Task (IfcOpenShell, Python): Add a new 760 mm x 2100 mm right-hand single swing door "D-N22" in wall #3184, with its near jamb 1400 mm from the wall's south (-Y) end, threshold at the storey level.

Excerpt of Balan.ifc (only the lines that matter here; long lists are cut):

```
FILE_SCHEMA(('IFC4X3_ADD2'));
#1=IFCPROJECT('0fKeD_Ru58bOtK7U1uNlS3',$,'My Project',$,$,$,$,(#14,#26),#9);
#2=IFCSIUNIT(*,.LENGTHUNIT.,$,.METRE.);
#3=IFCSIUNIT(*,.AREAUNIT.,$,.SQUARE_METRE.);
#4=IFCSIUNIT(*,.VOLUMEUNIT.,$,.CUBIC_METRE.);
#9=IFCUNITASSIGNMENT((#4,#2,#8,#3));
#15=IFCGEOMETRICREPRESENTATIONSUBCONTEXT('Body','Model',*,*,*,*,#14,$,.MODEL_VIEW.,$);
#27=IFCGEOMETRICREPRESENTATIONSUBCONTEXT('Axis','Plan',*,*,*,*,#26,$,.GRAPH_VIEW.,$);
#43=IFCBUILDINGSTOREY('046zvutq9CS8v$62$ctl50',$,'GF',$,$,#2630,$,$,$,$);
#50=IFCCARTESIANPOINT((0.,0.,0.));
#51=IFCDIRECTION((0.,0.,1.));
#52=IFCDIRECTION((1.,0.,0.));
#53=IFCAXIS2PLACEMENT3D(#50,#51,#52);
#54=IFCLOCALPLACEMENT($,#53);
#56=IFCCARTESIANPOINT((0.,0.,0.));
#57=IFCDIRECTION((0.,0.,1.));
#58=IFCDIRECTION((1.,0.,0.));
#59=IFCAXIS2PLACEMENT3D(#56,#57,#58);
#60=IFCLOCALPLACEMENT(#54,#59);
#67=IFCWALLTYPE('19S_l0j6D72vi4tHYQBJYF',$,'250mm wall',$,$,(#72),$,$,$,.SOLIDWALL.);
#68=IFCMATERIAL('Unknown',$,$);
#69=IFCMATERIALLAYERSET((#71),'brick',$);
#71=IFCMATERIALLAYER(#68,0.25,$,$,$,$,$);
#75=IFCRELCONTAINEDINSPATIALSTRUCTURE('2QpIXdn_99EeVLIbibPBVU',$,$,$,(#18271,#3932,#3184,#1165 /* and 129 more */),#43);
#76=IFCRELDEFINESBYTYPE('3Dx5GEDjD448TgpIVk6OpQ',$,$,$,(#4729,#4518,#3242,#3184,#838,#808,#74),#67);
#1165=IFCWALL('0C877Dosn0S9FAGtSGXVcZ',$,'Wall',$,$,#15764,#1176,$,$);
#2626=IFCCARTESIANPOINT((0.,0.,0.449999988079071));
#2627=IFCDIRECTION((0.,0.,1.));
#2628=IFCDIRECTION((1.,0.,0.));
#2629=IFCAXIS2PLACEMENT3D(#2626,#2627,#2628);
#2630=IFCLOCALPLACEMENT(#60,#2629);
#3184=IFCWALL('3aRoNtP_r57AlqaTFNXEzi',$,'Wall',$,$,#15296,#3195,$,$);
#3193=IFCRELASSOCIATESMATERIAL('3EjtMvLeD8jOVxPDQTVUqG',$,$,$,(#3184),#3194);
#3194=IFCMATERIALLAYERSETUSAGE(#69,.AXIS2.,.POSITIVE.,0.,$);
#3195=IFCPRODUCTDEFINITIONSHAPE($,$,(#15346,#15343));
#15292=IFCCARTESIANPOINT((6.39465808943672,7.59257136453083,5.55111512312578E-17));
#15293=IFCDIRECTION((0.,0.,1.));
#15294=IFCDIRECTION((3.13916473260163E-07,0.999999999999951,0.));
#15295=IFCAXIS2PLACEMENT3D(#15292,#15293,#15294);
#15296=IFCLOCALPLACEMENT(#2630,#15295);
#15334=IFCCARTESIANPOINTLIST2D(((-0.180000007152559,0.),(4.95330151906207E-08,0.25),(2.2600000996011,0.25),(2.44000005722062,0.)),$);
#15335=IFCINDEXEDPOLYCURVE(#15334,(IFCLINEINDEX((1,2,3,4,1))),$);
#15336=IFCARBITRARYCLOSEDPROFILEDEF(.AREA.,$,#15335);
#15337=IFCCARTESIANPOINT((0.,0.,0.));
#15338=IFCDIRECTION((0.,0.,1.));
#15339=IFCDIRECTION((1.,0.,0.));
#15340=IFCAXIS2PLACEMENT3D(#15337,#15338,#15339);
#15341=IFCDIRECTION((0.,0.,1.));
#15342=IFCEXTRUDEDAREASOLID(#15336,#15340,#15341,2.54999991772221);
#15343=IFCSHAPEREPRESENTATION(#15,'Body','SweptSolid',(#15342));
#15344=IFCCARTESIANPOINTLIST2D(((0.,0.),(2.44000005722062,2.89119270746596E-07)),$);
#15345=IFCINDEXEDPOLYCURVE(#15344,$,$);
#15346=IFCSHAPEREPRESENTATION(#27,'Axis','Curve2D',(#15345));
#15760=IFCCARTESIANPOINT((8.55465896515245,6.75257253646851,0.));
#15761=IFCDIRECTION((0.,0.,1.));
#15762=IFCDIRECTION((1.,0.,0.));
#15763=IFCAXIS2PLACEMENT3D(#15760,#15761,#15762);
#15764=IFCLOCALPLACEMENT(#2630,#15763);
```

```python
import numpy as np
import ifcopenshell
import ifcopenshell.api.feature
import ifcopenshell.api.geometry
import ifcopenshell.api.root
import ifcopenshell.api.spatial
import ifcopenshell.geom
import ifcopenshell.util.element
import ifcopenshell.util.placement
import ifcopenshell.util.representation
import ifcopenshell.util.shape
import ifcopenshell.util.unit

model = ifcopenshell.open("Balan.ifc")
unit_scale = ifcopenshell.util.unit.calculate_unit_scale(model)
settings = ifcopenshell.geom.settings()


def volume(element):
    """Net volume in cubic metres, openings subtracted."""
    shape = ifcopenshell.geom.create_shape(settings, element)
    return ifcopenshell.util.shape.get_volume(shape.geometry)


wall = model.by_guid("3aRoNtP_r57AlqaTFNXEzi")
storey = ifcopenshell.util.element.get_container(wall, ifc_class="IfcBuildingStorey")
context = ifcopenshell.util.representation.get_context(model, "Model", "Body", "MODEL_VIEW")
before = volume(wall)

width, height, from_end, sill = 0.76, 2.1, 1.4, 0.0  # metres

# The wall runs along its own X axis, and the end named is its -X end.
wall_shape = ifcopenshell.geom.create_shape(settings, wall)
x, y, z = ifcopenshell.util.shape.get_vertices(wall_shape.geometry).T
start = x.min() + from_end
face, thickness = float(y.min()), float(y.max() - y.min())
wall_matrix = ifcopenshell.util.placement.get_local_placement(wall.ObjectPlacement)
level = ifcopenshell.util.placement.get_local_placement(storey.ObjectPlacement)[2, 3]


def in_wall(x, y):
    """Placement at x, y metres in the wall's axes, at sill height."""
    matrix = wall_matrix.copy()
    matrix[:, 3] = wall_matrix @ np.array([x / unit_scale, y / unit_scale, 0.0, 1.0])
    matrix[2, 3] = level + sill / unit_scale
    return matrix


# Opening: a box that overshoots both wall faces by 50 mm.
opening = ifcopenshell.api.root.create_entity(model, ifc_class="IfcOpeningElement", predefined_type="OPENING")
box = ifcopenshell.api.geometry.add_wall_representation(
    model, context=context, length=width, height=height, thickness=thickness + 0.1
)
ifcopenshell.api.geometry.assign_representation(model, product=opening, representation=box)
ifcopenshell.api.geometry.edit_object_placement(model, product=opening, matrix=in_wall(start, face - 0.05), is_si=False)
ifcopenshell.api.feature.add_feature(model, feature=opening, element=wall)

door = ifcopenshell.api.root.create_entity(model, ifc_class="IfcDoor", name="D-N22", predefined_type="DOOR")
door.OverallWidth, door.OverallHeight = width / unit_scale, height / unit_scale
door.OperationType = "SINGLE_SWING_RIGHT"
body = ifcopenshell.api.geometry.add_door_representation(
    model,
    context=context,
    overall_width=door.OverallWidth,
    overall_height=door.OverallHeight,
    operation_type="SINGLE_SWING_RIGHT",
    lining_properties={"LiningDepth": thickness / unit_scale, "ThresholdDepth": thickness / unit_scale},
)
ifcopenshell.api.geometry.assign_representation(model, product=door, representation=body)
ifcopenshell.api.spatial.assign_container(model, products=[door], relating_structure=storey)
ifcopenshell.api.feature.add_filling(model, opening=opening, element=door)

# The lining spans the wall, so the door starts at the wall face.
ifcopenshell.api.geometry.edit_object_placement(model, product=door, matrix=in_wall(start, face), is_si=False)

after = volume(wall)

print(f"wall volume {before:.3f} -> {after:.3f} m3")

model.write("Balan_v2.ifc")
```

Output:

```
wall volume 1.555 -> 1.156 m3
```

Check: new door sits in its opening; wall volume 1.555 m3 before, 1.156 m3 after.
